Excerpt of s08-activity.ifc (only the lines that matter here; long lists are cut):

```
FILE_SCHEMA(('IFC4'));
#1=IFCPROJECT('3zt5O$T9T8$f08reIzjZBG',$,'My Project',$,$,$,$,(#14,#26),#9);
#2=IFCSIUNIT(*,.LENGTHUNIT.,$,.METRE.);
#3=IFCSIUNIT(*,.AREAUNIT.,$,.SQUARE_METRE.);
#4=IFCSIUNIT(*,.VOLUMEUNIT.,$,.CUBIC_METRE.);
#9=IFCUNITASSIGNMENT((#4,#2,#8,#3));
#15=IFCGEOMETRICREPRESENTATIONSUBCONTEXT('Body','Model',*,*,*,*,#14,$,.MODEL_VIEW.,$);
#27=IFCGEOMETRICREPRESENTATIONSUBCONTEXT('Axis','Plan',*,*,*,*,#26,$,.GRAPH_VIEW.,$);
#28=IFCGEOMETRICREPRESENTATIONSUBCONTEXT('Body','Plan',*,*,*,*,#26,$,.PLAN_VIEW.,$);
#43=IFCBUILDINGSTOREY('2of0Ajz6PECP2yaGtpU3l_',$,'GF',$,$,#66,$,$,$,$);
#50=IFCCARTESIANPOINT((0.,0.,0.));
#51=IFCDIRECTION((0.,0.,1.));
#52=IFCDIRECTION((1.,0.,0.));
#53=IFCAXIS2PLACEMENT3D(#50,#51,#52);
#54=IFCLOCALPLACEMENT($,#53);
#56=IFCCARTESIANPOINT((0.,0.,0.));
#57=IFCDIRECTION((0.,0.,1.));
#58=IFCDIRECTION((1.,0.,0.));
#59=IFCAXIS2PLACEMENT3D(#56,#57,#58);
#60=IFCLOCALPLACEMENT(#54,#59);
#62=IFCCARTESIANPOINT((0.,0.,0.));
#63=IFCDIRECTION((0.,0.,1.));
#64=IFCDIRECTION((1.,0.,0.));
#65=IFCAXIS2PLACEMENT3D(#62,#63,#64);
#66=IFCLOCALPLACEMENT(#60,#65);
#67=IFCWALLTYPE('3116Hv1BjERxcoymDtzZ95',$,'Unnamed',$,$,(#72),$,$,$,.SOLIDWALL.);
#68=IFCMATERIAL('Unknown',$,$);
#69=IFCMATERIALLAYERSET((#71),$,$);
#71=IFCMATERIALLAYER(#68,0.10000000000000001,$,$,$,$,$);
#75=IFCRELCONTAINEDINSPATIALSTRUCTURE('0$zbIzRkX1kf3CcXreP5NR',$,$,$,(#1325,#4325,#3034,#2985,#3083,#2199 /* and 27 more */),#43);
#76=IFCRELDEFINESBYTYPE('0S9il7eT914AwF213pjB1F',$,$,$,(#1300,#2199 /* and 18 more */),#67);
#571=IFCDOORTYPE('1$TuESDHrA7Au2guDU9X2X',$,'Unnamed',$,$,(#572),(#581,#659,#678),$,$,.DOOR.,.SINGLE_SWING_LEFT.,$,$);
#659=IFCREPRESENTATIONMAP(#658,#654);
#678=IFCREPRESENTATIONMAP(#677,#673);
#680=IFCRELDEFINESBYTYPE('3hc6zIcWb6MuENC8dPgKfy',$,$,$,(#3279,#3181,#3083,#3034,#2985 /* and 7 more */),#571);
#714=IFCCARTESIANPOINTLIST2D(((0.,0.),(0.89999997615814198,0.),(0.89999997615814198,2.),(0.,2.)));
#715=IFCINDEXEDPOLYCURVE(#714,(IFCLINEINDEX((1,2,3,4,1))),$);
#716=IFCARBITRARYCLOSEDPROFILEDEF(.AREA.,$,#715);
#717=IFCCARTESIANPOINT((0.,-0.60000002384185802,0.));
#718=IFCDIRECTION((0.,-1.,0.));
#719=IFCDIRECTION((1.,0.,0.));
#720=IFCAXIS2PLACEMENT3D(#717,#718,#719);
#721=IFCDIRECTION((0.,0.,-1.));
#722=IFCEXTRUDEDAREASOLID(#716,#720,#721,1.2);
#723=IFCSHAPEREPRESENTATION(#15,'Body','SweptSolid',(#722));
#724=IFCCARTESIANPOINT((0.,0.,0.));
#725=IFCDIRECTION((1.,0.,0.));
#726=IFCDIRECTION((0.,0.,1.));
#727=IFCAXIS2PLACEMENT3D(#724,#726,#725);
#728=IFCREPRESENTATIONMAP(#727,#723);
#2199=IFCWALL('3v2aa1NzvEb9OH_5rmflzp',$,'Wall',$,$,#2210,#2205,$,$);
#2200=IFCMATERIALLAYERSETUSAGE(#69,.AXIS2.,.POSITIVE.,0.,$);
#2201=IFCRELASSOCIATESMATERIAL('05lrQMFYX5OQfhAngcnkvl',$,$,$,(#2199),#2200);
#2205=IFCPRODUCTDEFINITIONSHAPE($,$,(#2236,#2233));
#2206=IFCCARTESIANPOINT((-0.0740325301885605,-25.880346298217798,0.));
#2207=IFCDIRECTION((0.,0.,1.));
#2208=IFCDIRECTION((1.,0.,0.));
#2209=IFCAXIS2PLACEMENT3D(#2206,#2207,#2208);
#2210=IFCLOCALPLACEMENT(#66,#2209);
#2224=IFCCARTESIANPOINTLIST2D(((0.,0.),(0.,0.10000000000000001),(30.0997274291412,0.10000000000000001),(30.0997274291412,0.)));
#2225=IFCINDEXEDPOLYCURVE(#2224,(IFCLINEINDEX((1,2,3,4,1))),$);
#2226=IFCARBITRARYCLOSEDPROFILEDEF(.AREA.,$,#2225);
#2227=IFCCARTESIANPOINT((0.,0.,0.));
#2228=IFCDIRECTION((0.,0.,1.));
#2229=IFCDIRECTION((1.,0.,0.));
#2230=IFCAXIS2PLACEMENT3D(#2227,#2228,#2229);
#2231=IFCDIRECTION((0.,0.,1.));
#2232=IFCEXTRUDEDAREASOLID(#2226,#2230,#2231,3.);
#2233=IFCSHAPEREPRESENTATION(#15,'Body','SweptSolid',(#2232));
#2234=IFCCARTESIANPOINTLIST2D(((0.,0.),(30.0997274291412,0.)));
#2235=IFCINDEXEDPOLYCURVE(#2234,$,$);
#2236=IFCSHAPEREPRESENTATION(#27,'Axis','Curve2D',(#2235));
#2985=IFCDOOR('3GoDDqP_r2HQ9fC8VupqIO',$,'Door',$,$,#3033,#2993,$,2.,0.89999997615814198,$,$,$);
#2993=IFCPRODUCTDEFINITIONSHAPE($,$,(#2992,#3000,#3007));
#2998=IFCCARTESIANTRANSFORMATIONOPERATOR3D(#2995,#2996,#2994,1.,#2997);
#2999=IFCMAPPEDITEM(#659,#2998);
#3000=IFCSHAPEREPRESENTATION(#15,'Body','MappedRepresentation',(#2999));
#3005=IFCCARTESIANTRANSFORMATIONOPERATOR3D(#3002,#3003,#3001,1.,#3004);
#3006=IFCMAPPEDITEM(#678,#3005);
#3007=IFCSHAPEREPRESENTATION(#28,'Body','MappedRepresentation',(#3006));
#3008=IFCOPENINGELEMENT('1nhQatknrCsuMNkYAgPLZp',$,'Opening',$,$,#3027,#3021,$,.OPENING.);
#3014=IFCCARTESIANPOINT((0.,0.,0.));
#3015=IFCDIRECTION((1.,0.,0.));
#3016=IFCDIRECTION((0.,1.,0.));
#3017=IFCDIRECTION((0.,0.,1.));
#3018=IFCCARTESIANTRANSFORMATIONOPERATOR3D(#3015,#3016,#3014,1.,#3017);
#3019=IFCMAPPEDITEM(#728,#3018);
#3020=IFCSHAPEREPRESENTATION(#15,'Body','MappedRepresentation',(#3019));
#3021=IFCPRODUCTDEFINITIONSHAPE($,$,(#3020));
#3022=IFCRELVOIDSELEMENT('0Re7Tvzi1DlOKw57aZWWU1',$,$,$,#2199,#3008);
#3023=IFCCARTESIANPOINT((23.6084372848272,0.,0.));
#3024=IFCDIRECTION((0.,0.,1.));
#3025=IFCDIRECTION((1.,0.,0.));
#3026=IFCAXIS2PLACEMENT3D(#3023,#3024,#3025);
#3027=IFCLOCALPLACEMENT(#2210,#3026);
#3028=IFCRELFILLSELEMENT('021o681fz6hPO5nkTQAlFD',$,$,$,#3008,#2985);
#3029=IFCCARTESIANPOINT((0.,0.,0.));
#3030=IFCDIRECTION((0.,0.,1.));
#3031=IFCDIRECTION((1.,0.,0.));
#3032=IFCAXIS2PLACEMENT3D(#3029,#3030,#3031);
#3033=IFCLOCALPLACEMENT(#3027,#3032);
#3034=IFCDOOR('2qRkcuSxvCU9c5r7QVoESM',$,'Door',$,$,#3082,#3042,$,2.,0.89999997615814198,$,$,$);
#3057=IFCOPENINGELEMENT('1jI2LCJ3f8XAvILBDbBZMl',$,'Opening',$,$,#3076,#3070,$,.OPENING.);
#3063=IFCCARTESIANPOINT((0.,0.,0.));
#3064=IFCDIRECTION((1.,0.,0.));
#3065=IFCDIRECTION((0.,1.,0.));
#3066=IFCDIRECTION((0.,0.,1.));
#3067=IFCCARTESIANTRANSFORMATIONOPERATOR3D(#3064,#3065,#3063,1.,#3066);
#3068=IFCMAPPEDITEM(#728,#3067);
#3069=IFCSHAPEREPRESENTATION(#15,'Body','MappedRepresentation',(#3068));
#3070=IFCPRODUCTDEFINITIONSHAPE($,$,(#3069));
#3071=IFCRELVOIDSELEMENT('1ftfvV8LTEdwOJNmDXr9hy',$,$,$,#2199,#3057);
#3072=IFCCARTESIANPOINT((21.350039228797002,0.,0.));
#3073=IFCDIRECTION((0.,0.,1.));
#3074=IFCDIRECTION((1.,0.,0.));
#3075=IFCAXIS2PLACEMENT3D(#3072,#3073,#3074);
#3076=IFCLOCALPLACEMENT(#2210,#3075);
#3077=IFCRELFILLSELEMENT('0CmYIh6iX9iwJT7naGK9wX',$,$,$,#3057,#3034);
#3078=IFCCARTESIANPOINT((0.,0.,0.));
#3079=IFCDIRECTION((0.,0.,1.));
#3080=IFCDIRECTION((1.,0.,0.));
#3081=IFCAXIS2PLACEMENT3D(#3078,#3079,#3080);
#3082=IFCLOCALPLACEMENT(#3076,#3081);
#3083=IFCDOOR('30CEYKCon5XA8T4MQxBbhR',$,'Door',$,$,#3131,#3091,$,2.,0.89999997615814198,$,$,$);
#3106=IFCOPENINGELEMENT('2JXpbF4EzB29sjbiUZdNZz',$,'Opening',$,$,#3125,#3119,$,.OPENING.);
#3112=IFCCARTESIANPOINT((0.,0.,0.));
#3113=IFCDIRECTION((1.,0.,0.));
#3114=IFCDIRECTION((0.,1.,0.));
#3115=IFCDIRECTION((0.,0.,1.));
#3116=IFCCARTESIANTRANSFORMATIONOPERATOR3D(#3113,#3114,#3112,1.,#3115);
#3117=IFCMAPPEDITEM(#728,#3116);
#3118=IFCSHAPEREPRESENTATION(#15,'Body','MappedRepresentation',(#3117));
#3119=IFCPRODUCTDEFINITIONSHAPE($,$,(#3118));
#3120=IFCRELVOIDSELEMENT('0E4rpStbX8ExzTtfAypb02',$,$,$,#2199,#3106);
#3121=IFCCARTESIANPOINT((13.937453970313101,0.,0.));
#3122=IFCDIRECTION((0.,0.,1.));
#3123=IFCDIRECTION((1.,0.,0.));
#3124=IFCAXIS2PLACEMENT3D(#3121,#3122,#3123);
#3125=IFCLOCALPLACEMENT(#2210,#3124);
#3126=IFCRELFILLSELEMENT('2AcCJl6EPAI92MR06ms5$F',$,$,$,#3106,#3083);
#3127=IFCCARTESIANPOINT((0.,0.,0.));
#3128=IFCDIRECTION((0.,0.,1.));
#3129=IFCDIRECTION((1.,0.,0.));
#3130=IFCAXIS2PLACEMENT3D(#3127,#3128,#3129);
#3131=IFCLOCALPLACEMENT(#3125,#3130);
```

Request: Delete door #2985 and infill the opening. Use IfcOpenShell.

```python
import ifcopenshell
import ifcopenshell.api.feature
import ifcopenshell.api.root
import ifcopenshell.geom
import ifcopenshell.util.shape

model = ifcopenshell.open("s08-activity.ifc")
settings = ifcopenshell.geom.settings()


def volume(element):
    """Net volume in cubic metres, openings subtracted."""
    shape = ifcopenshell.geom.create_shape(settings, element)
    return ifcopenshell.util.shape.get_volume(shape.geometry)


door = model.by_guid("3GoDDqP_r2HQ9fC8VupqIO")
opening = door.FillsVoids[0].RelatingOpeningElement
wall = opening.VoidsElements[0].RelatingBuildingElement
before = volume(wall)

ifcopenshell.api.root.remove_product(model, product=door)
ifcopenshell.api.feature.remove_feature(model, feature=opening)

after = volume(wall)

print(f"wall volume {before:.3f} -> {after:.3f} m3")

model.write("s08-activity_edited.ifc")
```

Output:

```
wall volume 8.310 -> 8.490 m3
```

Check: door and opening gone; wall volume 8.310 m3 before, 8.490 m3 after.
